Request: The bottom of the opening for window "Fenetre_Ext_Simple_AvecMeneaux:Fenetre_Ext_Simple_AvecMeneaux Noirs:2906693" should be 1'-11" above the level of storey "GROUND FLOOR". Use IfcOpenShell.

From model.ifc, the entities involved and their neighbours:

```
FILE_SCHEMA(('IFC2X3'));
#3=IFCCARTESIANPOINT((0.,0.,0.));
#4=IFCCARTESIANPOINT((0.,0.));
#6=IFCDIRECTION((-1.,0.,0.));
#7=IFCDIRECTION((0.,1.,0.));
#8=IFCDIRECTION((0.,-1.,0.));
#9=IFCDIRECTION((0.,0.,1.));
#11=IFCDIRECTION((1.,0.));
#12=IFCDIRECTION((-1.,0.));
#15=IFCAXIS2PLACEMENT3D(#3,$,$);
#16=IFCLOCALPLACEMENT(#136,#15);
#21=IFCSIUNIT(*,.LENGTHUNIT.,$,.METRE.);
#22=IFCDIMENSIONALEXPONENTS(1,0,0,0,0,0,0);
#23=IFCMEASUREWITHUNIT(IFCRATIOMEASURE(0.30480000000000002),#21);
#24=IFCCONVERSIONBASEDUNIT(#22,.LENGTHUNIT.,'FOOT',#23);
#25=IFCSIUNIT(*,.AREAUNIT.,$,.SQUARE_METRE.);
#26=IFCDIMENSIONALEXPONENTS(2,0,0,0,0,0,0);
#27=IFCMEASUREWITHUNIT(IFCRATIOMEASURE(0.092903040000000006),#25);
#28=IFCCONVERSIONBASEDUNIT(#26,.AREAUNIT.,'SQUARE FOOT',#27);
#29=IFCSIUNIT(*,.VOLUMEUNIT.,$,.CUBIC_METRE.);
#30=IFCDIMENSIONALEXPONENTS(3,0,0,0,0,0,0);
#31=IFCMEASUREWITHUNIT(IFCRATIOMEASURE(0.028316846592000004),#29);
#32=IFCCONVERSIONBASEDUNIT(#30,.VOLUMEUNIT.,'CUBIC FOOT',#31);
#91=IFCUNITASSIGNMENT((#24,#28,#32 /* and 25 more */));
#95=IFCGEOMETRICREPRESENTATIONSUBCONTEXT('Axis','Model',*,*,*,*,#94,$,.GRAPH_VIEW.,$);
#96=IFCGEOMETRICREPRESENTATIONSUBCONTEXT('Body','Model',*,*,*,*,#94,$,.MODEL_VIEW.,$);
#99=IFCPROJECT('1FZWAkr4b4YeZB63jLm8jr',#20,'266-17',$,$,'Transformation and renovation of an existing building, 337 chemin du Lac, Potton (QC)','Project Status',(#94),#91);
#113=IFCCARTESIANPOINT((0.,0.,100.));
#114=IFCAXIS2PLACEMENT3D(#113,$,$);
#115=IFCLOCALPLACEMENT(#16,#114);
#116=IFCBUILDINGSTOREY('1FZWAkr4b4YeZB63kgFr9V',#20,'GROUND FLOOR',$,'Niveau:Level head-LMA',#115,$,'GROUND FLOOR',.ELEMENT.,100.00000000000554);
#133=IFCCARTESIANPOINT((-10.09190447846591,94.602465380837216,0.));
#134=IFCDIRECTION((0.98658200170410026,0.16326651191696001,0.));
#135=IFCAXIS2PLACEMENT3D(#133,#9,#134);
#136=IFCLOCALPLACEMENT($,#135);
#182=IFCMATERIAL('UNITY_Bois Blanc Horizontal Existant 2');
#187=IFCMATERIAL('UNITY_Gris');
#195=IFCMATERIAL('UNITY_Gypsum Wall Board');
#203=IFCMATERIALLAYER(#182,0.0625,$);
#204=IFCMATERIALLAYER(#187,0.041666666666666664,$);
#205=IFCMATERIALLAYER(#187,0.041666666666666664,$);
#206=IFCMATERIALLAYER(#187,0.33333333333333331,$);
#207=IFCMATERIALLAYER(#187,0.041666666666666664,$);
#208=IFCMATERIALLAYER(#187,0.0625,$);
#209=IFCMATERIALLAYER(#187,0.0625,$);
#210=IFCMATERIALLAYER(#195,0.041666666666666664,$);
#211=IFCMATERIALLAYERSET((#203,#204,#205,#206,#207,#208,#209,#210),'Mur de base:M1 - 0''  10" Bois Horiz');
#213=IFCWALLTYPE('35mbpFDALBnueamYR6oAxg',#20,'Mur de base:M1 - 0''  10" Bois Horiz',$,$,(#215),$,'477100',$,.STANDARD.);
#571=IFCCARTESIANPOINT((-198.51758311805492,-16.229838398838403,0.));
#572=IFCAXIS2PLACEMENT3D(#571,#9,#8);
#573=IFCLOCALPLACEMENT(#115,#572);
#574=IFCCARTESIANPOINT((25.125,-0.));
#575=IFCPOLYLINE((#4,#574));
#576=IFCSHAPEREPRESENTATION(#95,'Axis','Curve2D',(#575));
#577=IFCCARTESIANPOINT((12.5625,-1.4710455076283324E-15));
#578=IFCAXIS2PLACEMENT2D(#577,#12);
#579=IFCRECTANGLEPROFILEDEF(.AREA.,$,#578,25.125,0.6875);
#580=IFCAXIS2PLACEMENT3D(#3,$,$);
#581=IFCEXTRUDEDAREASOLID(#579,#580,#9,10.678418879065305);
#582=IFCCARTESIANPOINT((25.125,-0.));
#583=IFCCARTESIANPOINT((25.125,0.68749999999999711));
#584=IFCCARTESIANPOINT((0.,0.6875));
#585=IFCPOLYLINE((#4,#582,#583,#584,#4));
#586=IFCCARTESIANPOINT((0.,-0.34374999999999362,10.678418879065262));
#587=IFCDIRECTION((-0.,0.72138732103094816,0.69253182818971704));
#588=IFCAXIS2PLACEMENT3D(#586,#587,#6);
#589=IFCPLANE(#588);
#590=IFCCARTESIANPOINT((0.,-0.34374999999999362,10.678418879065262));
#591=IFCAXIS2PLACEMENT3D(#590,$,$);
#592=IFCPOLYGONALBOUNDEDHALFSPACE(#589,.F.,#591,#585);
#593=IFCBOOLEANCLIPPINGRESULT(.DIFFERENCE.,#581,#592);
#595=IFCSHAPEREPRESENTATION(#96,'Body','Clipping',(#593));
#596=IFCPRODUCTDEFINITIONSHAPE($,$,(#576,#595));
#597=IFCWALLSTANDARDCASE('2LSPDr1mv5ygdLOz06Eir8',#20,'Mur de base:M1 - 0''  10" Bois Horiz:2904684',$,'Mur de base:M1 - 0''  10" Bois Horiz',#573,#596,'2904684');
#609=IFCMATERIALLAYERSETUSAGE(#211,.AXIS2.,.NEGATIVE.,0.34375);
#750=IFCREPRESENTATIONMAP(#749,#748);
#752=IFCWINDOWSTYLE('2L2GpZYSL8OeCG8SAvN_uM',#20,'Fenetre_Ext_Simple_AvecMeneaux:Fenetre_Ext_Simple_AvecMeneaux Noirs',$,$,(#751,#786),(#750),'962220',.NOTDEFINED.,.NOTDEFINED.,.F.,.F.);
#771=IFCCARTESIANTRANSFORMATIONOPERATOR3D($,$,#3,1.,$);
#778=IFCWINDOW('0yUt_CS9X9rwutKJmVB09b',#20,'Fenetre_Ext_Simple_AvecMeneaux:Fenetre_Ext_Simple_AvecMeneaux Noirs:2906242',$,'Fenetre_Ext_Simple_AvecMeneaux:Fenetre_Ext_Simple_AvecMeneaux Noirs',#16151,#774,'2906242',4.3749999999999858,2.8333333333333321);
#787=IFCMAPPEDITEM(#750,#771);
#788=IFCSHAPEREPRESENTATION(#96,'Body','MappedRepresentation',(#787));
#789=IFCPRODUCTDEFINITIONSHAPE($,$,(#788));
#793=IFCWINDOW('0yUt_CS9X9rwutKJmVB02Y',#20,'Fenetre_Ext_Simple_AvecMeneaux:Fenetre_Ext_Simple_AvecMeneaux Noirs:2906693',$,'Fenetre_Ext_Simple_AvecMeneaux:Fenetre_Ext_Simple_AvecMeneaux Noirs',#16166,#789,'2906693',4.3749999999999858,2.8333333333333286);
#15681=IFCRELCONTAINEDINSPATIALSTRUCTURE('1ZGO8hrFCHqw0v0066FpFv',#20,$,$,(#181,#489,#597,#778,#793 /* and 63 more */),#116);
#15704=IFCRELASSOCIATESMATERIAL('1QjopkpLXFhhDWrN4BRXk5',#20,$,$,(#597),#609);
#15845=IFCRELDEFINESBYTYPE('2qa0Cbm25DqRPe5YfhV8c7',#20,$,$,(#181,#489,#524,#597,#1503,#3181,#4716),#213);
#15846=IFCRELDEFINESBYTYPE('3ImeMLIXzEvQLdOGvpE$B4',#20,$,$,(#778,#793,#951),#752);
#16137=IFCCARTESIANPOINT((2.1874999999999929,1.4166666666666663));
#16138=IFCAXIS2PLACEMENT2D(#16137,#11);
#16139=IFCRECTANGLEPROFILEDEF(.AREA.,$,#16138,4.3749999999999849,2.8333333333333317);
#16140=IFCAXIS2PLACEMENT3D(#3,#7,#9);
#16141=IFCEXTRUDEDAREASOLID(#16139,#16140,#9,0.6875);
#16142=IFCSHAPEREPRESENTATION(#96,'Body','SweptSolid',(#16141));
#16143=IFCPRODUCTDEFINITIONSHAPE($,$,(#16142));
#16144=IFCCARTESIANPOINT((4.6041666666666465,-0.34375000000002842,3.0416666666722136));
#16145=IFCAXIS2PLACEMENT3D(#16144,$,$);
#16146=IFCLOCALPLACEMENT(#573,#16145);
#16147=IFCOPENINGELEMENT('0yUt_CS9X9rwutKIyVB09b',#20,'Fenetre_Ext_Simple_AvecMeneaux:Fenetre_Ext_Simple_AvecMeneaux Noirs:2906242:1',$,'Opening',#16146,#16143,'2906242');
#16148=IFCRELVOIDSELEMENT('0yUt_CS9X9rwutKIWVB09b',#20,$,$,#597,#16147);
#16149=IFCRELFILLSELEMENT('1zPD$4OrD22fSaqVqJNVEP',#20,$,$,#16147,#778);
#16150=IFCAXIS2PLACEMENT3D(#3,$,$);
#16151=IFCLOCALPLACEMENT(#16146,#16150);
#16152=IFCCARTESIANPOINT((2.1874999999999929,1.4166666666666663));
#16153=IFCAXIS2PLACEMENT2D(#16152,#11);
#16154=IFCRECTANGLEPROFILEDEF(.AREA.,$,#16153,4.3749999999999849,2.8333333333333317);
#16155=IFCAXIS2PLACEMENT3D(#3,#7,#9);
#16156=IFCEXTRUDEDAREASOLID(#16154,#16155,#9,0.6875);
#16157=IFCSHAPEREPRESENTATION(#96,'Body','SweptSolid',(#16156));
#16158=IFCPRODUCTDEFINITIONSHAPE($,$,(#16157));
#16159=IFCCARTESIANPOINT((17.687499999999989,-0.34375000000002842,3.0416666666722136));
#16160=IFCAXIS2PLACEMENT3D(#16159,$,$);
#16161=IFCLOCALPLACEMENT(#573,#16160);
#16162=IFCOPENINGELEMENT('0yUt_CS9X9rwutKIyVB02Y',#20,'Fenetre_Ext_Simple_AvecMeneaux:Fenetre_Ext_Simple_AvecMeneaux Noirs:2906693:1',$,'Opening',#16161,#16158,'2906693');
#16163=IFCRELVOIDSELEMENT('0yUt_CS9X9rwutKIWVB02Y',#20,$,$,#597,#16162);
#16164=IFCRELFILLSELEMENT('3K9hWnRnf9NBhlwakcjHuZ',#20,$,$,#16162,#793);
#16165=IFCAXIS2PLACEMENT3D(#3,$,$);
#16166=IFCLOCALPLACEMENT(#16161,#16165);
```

```python
import numpy as np
import ifcopenshell
import ifcopenshell.api.geometry
import ifcopenshell.geom
import ifcopenshell.util.element
import ifcopenshell.util.placement
import ifcopenshell.util.shape
import ifcopenshell.util.unit

model = ifcopenshell.open("model.ifc")
unit_scale = ifcopenshell.util.unit.calculate_unit_scale(model)

window = model.by_guid("0yUt_CS9X9rwutKJmVB02Y")
opening = window.FillsVoids[0].RelatingOpeningElement
storey = ifcopenshell.util.element.get_container(window, ifc_class="IfcBuildingStorey")
level = ifcopenshell.util.placement.get_local_placement(storey.ObjectPlacement)[2, 3]

# The opening's origin need not be at the sill, so measure its lowest point.
shape = ifcopenshell.geom.create_shape(ifcopenshell.geom.settings(), opening)
bottom = ifcopenshell.util.shape.get_shape_bottom_elevation(shape, shape.geometry) / unit_scale
dz = level + 23 * 0.0254 / unit_scale - bottom

shift = np.array([0.0, 0.0, dz])
# The window is placed relative to its opening, so it follows when the opening moves.
matrix = ifcopenshell.util.placement.get_local_placement(opening.ObjectPlacement)
matrix[:3, 3] += shift
ifcopenshell.api.geometry.edit_object_placement(
    model, product=opening, matrix=matrix, is_si=False, should_transform_children=True
)

print(f"moved by {dz * unit_scale:+.3f} m")

model.write("model_v2.ifc")
```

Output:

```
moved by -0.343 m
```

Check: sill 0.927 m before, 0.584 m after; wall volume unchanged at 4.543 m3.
